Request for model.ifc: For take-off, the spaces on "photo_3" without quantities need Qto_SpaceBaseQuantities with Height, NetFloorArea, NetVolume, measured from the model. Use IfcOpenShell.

First a look at what the model holds.

```python
import ifcopenshell
import ifcopenshell.util.element
import ifcopenshell.util.unit

model = ifcopenshell.open("model.ifc")
print(model.schema)
for unit_type in ("LENGTHUNIT", "AREAUNIT", "VOLUMEUNIT"):
    print(unit_type, ifcopenshell.util.unit.calculate_unit_scale(model, unit_type))
storey = next(s for s in model.by_type("IfcBuildingStorey") if s.Name == "photo_3")
spaces = [e for e in ifcopenshell.util.element.get_decomposition(storey) if e.is_a("IfcSpace")]
for e in sorted(spaces, key=lambda e: e.id()):
    print(e.id(), e.is_a(), e.Name, list(ifcopenshell.util.element.get_psets(e, qtos_only=True)), sep=" | ")
```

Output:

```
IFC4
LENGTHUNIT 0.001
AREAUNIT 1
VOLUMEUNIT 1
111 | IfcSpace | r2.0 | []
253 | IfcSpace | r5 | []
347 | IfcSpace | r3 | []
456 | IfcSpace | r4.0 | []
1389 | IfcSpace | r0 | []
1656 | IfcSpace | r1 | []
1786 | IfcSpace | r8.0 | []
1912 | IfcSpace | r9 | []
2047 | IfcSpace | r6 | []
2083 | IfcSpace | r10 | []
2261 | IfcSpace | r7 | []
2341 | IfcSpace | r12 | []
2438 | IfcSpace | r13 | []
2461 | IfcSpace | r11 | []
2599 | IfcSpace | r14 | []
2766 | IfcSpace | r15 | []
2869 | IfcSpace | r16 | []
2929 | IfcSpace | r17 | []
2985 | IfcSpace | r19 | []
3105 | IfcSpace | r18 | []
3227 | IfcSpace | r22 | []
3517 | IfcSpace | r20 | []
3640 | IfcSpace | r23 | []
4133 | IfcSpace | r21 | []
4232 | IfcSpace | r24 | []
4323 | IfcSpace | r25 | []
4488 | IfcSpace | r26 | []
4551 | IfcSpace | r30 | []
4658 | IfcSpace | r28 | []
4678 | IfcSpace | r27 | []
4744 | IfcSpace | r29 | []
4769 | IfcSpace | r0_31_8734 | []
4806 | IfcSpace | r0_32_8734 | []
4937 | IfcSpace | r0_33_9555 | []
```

```python
import ifcopenshell
import ifcopenshell.api.pset
import ifcopenshell.geom
import ifcopenshell.util.element
import ifcopenshell.util.shape
import ifcopenshell.util.unit

model = ifcopenshell.open("model.ifc")
unit_scale = ifcopenshell.util.unit.calculate_unit_scale(model)
area_scale = ifcopenshell.util.unit.calculate_unit_scale(model, "AREAUNIT")
volume_scale = ifcopenshell.util.unit.calculate_unit_scale(model, "VOLUMEUNIT")
settings = ifcopenshell.geom.settings()

storey = next(s for s in model.by_type("IfcBuildingStorey") if s.Name == "photo_3")
spaces = [e for e in ifcopenshell.util.element.get_decomposition(storey) if e.is_a("IfcSpace")]

for e in sorted(spaces, key=lambda e: e.id()):
    if ifcopenshell.util.element.get_psets(e, qtos_only=True, should_inherit=False):
        continue
    # Geometry comes back in metres, in the element's own axes.
    shape = ifcopenshell.geom.create_shape(settings, e)
    values = {
        "Height": ifcopenshell.util.shape.get_z(shape.geometry) / unit_scale,
        "NetFloorArea": ifcopenshell.util.shape.get_footprint_area(shape.geometry) / area_scale,
        "NetVolume": ifcopenshell.util.shape.get_volume(shape.geometry) / volume_scale,
    }
    qto = ifcopenshell.api.pset.add_qto(model, product=e, name="Qto_SpaceBaseQuantities")
    ifcopenshell.api.pset.edit_qto(model, qto=qto, properties=values)
    print(e.id(), {k: round(v, 3) for k, v in values.items()})

model.write("model_updated.ifc")
```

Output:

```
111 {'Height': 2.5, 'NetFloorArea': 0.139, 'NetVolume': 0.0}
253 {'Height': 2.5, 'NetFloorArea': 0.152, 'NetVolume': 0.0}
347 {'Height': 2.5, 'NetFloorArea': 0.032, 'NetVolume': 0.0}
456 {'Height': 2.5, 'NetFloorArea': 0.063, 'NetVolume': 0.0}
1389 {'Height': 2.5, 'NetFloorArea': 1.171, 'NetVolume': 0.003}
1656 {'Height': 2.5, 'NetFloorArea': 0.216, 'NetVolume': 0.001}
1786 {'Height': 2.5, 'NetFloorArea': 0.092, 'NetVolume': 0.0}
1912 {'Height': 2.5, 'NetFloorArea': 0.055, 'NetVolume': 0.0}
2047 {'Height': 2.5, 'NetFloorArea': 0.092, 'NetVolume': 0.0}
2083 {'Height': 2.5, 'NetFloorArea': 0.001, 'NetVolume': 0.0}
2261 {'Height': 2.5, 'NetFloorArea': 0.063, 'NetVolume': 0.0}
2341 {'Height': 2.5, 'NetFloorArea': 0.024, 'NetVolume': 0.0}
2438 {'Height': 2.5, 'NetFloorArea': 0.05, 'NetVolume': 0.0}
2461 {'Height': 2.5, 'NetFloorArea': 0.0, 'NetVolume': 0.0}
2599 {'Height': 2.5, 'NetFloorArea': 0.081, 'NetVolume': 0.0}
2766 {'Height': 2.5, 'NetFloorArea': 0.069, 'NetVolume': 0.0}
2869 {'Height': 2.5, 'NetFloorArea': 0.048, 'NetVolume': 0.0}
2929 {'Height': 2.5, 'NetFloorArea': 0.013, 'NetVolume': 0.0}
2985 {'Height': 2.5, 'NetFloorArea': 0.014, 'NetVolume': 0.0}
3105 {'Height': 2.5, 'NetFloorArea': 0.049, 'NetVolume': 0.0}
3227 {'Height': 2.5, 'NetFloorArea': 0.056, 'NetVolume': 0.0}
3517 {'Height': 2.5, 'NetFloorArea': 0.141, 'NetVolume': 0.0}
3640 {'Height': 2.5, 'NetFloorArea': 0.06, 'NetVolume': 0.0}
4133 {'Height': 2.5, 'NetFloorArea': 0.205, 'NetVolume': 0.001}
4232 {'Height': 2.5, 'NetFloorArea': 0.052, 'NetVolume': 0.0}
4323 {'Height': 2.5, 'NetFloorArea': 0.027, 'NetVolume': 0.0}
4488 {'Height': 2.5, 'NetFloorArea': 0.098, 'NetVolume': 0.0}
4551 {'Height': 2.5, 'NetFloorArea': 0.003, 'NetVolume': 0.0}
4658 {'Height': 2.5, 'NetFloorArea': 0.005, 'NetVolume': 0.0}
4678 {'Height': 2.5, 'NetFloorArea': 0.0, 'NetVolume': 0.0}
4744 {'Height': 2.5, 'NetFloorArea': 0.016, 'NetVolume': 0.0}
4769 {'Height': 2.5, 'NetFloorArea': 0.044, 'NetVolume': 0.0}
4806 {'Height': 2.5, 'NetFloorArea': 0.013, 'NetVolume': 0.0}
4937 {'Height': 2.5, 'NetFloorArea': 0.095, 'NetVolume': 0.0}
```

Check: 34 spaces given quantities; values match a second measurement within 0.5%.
